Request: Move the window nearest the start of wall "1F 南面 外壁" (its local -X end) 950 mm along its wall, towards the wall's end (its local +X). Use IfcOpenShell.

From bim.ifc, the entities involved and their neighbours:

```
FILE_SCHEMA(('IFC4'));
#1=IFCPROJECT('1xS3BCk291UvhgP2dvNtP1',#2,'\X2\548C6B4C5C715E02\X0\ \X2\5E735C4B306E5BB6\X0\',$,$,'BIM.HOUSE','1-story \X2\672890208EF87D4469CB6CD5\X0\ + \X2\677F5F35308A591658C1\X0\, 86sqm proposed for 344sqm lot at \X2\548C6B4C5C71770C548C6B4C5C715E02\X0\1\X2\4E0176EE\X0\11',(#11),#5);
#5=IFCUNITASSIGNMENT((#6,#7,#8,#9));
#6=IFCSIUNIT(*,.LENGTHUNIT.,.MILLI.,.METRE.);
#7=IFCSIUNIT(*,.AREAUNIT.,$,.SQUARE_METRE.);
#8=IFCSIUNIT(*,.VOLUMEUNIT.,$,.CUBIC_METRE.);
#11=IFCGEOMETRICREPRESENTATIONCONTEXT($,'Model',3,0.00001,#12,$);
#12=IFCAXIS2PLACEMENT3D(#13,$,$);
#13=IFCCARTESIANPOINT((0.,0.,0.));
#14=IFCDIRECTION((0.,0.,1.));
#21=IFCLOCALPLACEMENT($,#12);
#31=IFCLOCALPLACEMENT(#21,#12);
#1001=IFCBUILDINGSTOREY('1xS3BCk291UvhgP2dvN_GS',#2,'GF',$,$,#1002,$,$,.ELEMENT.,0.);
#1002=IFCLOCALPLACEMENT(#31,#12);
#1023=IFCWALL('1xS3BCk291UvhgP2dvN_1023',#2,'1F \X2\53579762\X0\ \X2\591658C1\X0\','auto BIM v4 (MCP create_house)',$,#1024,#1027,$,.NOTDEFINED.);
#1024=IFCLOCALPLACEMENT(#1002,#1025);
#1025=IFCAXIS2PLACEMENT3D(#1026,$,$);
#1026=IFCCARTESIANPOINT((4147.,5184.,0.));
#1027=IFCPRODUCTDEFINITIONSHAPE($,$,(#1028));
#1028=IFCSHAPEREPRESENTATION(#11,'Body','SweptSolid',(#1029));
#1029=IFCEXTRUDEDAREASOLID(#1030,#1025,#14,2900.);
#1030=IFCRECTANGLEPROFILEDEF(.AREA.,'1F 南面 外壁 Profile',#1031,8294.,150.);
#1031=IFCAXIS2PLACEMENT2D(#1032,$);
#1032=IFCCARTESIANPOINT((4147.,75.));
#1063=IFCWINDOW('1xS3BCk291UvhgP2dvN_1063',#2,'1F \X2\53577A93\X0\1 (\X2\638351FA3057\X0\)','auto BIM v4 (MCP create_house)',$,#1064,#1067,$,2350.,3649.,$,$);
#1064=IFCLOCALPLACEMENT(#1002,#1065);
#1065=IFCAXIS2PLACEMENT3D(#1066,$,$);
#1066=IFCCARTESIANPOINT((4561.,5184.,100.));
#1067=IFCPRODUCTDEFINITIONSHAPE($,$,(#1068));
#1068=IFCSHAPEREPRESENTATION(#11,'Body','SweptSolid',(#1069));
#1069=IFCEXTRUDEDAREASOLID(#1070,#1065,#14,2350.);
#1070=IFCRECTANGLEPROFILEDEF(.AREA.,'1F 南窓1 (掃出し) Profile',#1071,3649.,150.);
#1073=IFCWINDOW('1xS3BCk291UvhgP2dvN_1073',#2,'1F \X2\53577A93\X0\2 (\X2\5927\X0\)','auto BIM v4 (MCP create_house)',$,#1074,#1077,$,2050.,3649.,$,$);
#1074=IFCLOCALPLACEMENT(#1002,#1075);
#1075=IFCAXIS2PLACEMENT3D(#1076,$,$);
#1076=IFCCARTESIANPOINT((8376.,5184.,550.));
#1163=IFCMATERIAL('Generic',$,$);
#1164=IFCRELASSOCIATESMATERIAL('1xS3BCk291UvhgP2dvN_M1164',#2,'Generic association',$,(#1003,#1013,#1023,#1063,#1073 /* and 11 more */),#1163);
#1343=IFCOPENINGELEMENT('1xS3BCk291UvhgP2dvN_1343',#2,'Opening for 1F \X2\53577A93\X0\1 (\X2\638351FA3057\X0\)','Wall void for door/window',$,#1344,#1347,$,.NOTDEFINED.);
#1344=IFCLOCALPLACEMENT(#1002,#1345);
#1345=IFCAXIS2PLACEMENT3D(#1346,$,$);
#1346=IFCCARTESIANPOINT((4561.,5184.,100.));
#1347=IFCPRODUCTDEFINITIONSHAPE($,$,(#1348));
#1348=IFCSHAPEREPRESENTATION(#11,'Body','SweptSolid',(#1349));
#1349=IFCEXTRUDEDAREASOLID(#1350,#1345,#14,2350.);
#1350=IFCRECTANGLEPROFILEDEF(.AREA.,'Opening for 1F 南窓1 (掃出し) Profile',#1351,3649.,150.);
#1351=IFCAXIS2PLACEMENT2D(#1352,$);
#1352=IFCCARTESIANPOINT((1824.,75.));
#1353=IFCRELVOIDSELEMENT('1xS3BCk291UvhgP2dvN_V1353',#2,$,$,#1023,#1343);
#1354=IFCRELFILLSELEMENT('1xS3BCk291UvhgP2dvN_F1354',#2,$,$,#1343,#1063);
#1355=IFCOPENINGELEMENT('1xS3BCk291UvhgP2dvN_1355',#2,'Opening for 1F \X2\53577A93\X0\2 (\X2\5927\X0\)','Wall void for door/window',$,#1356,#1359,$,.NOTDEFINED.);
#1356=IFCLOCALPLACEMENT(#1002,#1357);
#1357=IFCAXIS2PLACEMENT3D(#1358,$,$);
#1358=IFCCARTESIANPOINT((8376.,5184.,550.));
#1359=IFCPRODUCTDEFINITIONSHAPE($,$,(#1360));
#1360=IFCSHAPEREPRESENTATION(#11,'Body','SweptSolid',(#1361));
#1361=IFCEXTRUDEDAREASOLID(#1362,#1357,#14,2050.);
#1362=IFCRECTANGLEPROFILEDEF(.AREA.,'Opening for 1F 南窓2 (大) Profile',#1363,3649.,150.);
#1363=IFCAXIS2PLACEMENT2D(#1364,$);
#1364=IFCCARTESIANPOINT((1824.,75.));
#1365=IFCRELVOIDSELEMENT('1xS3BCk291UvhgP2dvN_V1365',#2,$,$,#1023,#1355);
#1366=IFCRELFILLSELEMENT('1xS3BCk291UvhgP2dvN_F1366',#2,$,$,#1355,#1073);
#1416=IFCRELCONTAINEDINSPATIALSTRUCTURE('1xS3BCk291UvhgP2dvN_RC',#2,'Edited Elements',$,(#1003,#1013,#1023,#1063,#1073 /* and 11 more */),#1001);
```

```python
import ifcopenshell
import ifcopenshell.api.geometry
import ifcopenshell.util.placement
import ifcopenshell.util.unit

model = ifcopenshell.open("bim.ifc")
unit_scale = ifcopenshell.util.unit.calculate_unit_scale(model)

window = model.by_guid("1xS3BCk291UvhgP2dvN_1063")
opening = window.FillsVoids[0].RelatingOpeningElement
wall = opening.VoidsElements[0].RelatingBuildingElement

wall_matrix = ifcopenshell.util.placement.get_local_placement(wall.ObjectPlacement)
shift = wall_matrix[:3, 0] * 0.95 / unit_scale
before = ifcopenshell.util.placement.get_local_placement(window.ObjectPlacement)[:3, 3].copy()

# The window is not placed relative to its opening, so move both.
for product in (opening, window):
    matrix = ifcopenshell.util.placement.get_local_placement(product.ObjectPlacement)
    matrix[:3, 3] += shift
    ifcopenshell.api.geometry.edit_object_placement(model, product=product, matrix=matrix, is_si=False)

after = ifcopenshell.util.placement.get_local_placement(window.ObjectPlacement)[:3, 3]
print("window moved by", (after - before).round(3) + 0.0)

model.write("bim_edited.ifc")
```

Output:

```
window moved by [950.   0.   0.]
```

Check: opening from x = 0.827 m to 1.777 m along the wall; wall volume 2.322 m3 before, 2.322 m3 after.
